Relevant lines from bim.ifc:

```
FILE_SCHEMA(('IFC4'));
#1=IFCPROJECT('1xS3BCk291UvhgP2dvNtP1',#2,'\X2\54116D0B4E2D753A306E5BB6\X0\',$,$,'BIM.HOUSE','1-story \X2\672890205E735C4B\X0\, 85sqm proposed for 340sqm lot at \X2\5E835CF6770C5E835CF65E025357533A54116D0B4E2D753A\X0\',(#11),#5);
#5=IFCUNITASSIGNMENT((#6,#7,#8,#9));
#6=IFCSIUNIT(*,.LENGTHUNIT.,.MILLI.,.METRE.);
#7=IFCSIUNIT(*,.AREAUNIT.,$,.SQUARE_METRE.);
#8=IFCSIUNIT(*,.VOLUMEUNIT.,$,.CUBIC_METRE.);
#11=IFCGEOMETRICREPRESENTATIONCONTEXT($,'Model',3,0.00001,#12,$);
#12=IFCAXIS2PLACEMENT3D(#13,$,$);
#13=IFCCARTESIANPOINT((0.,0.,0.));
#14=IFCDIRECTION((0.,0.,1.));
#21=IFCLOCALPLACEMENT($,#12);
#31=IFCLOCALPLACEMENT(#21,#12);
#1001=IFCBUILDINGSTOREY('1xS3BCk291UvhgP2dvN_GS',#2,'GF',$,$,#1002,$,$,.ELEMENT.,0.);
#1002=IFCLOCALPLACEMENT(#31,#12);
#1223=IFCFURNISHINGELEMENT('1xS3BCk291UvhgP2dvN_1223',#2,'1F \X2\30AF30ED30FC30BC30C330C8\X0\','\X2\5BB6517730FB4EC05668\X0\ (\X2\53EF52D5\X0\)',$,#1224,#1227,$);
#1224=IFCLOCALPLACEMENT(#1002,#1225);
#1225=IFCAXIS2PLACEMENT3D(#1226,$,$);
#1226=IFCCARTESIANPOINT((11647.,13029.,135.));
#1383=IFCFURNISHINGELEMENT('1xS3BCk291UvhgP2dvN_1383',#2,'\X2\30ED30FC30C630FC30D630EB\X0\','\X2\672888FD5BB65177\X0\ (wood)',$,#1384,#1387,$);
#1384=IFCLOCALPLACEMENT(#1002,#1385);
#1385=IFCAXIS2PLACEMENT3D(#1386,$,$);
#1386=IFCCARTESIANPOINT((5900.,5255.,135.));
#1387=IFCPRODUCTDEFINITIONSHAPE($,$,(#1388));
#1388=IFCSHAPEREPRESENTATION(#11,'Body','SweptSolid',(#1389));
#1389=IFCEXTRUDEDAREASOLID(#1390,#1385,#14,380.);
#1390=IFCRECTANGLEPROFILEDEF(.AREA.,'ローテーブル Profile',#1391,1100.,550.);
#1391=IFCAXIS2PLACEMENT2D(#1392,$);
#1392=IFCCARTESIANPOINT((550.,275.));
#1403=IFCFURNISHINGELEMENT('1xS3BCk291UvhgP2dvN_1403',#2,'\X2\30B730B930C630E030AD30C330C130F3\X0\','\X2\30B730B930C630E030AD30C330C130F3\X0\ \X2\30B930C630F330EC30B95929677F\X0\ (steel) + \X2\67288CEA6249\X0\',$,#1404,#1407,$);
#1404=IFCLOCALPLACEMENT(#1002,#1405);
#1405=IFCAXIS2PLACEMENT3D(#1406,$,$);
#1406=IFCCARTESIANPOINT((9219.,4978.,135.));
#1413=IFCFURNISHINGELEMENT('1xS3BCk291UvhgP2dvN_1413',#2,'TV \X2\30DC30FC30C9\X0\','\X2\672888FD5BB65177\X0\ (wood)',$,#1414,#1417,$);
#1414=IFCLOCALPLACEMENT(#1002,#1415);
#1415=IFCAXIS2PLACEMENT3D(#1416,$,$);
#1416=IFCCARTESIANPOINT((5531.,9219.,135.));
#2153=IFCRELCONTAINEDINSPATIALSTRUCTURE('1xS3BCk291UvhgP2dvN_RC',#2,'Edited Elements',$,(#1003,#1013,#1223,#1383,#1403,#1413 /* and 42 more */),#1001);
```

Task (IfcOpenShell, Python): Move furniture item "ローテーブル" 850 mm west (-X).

```python
import ifcopenshell
import ifcopenshell.api.geometry
import ifcopenshell.util.placement

model = ifcopenshell.open("bim.ifc")

item = model.by_guid("1xS3BCk291UvhgP2dvN_1383")
matrix = ifcopenshell.util.placement.get_local_placement(item.ObjectPlacement)
matrix[0, 3] -= 850.0
ifcopenshell.api.geometry.edit_object_placement(model, product=item, matrix=matrix, is_si=False)

print(ifcopenshell.util.placement.get_local_placement(item.ObjectPlacement).round(3) + 0.0)

model.write("bim_v2.ifc")
```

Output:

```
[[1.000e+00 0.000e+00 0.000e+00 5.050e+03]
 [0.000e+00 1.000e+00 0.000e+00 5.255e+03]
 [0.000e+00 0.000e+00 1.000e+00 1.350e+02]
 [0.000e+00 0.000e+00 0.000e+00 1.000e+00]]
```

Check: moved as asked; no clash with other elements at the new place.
